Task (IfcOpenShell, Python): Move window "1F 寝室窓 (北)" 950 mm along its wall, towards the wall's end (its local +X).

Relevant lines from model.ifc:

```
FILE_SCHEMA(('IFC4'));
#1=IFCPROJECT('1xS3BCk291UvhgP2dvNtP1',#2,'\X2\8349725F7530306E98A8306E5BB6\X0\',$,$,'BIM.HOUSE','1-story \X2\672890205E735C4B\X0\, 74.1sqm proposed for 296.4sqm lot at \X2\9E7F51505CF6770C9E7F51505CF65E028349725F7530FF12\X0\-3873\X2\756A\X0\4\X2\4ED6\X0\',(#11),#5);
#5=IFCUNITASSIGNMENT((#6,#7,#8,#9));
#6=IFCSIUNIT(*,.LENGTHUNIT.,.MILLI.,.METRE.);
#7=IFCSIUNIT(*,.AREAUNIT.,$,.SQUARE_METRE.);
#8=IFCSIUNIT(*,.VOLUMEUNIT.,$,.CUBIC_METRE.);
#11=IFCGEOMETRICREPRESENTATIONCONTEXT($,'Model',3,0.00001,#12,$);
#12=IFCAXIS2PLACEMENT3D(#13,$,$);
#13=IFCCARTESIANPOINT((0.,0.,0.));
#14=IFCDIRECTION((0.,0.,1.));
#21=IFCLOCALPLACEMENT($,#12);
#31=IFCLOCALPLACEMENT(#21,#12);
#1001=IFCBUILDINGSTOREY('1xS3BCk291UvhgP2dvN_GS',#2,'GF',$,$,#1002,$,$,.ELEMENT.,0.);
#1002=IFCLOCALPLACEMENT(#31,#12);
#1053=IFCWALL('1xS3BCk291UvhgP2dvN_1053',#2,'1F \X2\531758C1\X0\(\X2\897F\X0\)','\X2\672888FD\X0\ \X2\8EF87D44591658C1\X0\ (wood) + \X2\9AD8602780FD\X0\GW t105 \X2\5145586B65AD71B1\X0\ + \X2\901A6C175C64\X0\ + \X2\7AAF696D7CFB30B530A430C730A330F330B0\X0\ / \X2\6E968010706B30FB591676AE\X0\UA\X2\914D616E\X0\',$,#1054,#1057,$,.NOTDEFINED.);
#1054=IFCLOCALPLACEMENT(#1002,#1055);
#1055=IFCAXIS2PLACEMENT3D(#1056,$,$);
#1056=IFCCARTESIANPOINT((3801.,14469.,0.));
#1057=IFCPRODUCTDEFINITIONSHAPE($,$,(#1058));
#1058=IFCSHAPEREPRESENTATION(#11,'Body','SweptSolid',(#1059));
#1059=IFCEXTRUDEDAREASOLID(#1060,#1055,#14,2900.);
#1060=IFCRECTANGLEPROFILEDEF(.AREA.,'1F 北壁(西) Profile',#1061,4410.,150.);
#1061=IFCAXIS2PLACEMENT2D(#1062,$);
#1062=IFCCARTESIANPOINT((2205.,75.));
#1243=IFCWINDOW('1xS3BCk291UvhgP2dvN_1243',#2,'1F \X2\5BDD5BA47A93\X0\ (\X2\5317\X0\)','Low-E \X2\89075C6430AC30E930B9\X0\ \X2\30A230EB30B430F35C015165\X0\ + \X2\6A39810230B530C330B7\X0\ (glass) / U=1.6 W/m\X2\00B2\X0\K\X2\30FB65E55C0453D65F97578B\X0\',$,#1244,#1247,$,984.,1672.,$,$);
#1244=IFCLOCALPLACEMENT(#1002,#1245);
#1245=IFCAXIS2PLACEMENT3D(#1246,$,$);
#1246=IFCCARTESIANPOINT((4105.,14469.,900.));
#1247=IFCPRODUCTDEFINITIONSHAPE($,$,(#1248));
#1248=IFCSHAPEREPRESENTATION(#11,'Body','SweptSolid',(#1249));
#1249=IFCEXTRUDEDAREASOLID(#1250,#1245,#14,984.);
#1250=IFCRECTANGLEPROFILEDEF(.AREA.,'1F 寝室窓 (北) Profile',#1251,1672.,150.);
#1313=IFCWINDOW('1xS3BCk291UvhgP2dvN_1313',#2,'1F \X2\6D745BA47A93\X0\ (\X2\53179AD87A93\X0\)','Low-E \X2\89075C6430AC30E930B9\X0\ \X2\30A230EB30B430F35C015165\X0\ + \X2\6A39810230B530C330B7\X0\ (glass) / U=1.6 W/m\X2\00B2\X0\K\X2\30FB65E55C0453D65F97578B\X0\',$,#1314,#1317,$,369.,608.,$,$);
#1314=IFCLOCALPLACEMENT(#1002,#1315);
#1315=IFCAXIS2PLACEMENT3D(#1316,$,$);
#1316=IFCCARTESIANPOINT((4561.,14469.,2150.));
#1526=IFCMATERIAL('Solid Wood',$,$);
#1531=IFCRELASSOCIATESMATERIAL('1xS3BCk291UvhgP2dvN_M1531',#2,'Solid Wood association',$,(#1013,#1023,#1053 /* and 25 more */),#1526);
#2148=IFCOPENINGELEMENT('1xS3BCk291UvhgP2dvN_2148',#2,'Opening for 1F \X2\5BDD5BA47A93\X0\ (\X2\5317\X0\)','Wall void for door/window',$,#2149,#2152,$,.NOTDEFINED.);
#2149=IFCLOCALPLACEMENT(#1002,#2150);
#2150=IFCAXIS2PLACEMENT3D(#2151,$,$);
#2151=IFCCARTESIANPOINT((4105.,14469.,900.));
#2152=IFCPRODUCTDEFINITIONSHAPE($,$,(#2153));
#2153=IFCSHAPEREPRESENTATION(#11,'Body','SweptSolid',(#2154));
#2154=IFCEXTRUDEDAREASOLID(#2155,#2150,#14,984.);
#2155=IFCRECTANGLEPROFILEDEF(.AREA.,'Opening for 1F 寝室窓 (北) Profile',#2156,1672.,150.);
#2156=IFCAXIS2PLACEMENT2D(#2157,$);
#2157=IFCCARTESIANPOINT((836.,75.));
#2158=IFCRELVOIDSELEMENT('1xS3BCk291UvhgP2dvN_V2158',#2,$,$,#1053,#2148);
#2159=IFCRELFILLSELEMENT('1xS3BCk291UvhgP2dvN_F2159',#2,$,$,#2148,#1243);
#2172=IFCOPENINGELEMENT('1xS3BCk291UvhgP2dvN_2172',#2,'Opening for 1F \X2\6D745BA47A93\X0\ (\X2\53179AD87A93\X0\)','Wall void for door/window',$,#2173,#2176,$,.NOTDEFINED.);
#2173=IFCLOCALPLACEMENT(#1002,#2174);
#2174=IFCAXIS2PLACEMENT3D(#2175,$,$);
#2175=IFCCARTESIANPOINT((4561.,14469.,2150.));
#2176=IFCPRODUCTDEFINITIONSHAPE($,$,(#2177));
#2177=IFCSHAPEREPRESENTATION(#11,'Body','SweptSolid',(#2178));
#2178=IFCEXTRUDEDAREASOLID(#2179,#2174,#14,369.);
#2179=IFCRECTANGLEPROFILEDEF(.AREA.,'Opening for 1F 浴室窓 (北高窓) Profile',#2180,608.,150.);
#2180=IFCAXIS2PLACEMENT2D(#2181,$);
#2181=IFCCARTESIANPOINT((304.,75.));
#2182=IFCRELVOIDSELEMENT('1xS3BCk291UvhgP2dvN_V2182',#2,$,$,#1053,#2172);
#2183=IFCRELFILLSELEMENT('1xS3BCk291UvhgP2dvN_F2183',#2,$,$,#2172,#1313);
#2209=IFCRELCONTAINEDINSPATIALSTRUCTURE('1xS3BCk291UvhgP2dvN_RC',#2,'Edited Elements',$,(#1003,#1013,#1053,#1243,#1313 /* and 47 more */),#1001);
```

```python
import ifcopenshell
import ifcopenshell.api.geometry
import ifcopenshell.util.placement
import ifcopenshell.util.unit

model = ifcopenshell.open("model.ifc")
unit_scale = ifcopenshell.util.unit.calculate_unit_scale(model)

window = model.by_guid("1xS3BCk291UvhgP2dvN_1243")
opening = window.FillsVoids[0].RelatingOpeningElement
wall = opening.VoidsElements[0].RelatingBuildingElement

wall_matrix = ifcopenshell.util.placement.get_local_placement(wall.ObjectPlacement)
shift = wall_matrix[:3, 0] * 0.95 / unit_scale
before = ifcopenshell.util.placement.get_local_placement(window.ObjectPlacement)[:3, 3].copy()

# The window is not placed relative to its opening, so move both.
for product in (opening, window):
    matrix = ifcopenshell.util.placement.get_local_placement(product.ObjectPlacement)
    matrix[:3, 3] += shift
    ifcopenshell.api.geometry.edit_object_placement(model, product=product, matrix=matrix, is_si=False)

after = ifcopenshell.util.placement.get_local_placement(window.ObjectPlacement)[:3, 3]
print("window moved by", (after - before).round(3) + 0.0)

model.write("model_v2.ifc")
```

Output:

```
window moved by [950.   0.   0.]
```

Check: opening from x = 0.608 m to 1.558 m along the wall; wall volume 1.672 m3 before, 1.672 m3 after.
